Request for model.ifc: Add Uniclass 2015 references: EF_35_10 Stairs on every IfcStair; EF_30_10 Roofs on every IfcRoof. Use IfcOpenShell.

First a look at what the model holds.

```python
import ifcopenshell

model = ifcopenshell.open("model.ifc")
print(model.schema)
print("classifications:", [c.Name for c in model.by_type("IfcClassification")])
for ifc_class in ("IfcDoor", "IfcRoof", "IfcStair", "IfcWall", "IfcWindow"):
    print(ifc_class, len(model.by_type(ifc_class)))
```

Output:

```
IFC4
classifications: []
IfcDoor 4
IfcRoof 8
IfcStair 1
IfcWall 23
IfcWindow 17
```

```python
import ifcopenshell
import ifcopenshell.api.classification

model = ifcopenshell.open("model.ifc")

system = ifcopenshell.api.classification.add_classification(model, classification="Uniclass 2015")

codes = {
    "IfcStair": ("EF_35_10", "Stairs"),
    "IfcRoof": ("EF_30_10", "Roofs"),
}
for ifc_class, (code, name) in codes.items():
    products = model.by_type(ifc_class)
    ifcopenshell.api.classification.add_reference(
        model, products=products, classification=system, identification=code, name=name
    )
    print(code, len(products))

model.write("model_rev.ifc")
```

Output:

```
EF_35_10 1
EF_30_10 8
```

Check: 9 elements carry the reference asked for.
